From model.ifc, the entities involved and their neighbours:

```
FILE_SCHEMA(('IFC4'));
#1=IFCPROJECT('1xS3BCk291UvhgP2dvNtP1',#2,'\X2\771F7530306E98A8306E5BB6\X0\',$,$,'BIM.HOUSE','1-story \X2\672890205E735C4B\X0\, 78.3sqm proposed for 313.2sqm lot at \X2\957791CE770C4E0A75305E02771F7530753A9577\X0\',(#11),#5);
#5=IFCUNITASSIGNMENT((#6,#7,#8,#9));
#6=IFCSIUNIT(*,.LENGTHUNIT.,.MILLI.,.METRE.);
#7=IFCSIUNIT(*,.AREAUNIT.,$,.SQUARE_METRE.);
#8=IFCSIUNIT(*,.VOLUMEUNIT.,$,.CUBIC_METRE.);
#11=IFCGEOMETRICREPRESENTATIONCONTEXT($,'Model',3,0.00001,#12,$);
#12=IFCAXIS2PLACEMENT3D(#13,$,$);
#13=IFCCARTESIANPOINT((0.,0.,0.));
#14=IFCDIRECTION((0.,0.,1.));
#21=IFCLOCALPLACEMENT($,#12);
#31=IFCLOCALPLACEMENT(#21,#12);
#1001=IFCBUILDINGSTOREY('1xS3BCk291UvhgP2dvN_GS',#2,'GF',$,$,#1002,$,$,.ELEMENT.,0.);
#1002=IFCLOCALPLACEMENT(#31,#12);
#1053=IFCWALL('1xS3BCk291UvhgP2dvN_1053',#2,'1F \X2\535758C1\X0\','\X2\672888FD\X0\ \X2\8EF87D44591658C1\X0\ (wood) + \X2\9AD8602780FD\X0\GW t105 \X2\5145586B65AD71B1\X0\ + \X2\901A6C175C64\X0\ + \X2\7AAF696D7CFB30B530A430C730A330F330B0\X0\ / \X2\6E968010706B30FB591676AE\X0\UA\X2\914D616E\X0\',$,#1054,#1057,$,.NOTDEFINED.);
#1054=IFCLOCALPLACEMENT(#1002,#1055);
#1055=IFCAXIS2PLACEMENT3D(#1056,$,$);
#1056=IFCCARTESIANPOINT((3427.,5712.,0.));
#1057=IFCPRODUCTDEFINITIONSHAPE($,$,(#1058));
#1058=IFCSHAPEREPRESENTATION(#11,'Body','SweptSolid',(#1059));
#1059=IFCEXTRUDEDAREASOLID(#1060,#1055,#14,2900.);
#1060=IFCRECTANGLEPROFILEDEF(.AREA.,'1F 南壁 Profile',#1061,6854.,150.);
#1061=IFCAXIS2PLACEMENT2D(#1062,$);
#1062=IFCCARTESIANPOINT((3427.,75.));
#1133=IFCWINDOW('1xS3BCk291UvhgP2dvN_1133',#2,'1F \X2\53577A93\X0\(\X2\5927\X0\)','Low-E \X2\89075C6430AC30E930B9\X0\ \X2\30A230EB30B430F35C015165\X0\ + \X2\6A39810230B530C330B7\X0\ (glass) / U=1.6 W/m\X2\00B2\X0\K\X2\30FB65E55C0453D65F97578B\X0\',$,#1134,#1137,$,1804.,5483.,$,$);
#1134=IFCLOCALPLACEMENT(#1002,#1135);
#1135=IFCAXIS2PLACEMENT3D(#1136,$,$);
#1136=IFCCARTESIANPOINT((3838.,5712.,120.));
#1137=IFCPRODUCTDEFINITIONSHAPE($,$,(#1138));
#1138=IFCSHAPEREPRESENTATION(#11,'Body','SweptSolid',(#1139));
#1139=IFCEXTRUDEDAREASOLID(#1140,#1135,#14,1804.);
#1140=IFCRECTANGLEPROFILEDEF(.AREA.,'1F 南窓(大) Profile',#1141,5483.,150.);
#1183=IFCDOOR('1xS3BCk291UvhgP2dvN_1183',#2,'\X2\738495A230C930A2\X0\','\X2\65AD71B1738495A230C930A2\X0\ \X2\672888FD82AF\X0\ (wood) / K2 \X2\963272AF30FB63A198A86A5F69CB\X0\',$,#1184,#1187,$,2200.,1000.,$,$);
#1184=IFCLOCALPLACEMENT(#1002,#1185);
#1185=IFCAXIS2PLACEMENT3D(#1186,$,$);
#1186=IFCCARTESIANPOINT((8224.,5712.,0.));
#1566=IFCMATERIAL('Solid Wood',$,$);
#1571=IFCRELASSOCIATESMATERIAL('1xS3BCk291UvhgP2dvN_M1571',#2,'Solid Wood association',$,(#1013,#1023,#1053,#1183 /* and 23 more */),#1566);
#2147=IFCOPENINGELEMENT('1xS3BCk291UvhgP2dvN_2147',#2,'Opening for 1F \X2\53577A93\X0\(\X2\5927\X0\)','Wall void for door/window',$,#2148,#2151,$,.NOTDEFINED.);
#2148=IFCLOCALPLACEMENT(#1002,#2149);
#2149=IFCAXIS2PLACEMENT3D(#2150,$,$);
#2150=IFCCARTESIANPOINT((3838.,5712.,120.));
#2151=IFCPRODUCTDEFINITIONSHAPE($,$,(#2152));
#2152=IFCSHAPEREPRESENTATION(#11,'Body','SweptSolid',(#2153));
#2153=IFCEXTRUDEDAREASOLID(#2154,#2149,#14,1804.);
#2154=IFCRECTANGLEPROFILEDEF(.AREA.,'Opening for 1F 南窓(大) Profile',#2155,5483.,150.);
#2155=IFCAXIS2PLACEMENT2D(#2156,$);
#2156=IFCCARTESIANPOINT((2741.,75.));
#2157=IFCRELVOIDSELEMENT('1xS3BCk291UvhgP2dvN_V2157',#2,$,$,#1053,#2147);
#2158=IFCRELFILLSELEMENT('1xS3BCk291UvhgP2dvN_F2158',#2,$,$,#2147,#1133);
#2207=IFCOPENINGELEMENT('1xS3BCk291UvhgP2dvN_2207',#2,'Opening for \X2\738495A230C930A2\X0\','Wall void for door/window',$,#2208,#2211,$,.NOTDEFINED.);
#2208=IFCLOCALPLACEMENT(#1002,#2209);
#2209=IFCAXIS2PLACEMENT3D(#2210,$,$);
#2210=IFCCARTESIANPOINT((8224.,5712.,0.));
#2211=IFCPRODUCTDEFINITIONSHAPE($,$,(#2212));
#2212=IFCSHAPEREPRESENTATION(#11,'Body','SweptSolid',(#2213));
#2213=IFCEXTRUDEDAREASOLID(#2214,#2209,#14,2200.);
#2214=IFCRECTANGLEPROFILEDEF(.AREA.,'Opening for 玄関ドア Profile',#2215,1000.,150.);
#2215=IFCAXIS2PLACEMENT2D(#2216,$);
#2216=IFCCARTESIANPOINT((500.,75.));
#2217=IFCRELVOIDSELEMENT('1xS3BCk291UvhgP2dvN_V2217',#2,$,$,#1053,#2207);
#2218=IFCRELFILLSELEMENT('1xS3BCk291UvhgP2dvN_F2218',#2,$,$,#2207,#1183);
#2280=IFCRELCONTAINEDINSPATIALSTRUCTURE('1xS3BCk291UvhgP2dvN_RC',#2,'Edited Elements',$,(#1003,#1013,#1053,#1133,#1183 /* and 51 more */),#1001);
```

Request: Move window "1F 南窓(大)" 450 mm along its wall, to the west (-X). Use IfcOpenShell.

```python
import ifcopenshell
import ifcopenshell.api.geometry
import ifcopenshell.util.placement
import ifcopenshell.util.unit

model = ifcopenshell.open("model.ifc")
unit_scale = ifcopenshell.util.unit.calculate_unit_scale(model)

window = model.by_id(1133)
opening = window.FillsVoids[0].RelatingOpeningElement
wall = opening.VoidsElements[0].RelatingBuildingElement

wall_matrix = ifcopenshell.util.placement.get_local_placement(wall.ObjectPlacement)
shift = wall_matrix[:3, 0] * -0.45 / unit_scale
before = ifcopenshell.util.placement.get_local_placement(window.ObjectPlacement)[:3, 3].copy()

# The window is not placed relative to its opening, so move both.
for product in (opening, window):
    matrix = ifcopenshell.util.placement.get_local_placement(product.ObjectPlacement)
    matrix[:3, 3] += shift
    ifcopenshell.api.geometry.edit_object_placement(model, product=product, matrix=matrix, is_si=False)

after = ifcopenshell.util.placement.get_local_placement(window.ObjectPlacement)[:3, 3]
print("window moved by", (after - before).round(3) + 0.0)

model.write("model_edited.ifc")
```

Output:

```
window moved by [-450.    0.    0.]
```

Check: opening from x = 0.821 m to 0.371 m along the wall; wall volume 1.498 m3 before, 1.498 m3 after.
